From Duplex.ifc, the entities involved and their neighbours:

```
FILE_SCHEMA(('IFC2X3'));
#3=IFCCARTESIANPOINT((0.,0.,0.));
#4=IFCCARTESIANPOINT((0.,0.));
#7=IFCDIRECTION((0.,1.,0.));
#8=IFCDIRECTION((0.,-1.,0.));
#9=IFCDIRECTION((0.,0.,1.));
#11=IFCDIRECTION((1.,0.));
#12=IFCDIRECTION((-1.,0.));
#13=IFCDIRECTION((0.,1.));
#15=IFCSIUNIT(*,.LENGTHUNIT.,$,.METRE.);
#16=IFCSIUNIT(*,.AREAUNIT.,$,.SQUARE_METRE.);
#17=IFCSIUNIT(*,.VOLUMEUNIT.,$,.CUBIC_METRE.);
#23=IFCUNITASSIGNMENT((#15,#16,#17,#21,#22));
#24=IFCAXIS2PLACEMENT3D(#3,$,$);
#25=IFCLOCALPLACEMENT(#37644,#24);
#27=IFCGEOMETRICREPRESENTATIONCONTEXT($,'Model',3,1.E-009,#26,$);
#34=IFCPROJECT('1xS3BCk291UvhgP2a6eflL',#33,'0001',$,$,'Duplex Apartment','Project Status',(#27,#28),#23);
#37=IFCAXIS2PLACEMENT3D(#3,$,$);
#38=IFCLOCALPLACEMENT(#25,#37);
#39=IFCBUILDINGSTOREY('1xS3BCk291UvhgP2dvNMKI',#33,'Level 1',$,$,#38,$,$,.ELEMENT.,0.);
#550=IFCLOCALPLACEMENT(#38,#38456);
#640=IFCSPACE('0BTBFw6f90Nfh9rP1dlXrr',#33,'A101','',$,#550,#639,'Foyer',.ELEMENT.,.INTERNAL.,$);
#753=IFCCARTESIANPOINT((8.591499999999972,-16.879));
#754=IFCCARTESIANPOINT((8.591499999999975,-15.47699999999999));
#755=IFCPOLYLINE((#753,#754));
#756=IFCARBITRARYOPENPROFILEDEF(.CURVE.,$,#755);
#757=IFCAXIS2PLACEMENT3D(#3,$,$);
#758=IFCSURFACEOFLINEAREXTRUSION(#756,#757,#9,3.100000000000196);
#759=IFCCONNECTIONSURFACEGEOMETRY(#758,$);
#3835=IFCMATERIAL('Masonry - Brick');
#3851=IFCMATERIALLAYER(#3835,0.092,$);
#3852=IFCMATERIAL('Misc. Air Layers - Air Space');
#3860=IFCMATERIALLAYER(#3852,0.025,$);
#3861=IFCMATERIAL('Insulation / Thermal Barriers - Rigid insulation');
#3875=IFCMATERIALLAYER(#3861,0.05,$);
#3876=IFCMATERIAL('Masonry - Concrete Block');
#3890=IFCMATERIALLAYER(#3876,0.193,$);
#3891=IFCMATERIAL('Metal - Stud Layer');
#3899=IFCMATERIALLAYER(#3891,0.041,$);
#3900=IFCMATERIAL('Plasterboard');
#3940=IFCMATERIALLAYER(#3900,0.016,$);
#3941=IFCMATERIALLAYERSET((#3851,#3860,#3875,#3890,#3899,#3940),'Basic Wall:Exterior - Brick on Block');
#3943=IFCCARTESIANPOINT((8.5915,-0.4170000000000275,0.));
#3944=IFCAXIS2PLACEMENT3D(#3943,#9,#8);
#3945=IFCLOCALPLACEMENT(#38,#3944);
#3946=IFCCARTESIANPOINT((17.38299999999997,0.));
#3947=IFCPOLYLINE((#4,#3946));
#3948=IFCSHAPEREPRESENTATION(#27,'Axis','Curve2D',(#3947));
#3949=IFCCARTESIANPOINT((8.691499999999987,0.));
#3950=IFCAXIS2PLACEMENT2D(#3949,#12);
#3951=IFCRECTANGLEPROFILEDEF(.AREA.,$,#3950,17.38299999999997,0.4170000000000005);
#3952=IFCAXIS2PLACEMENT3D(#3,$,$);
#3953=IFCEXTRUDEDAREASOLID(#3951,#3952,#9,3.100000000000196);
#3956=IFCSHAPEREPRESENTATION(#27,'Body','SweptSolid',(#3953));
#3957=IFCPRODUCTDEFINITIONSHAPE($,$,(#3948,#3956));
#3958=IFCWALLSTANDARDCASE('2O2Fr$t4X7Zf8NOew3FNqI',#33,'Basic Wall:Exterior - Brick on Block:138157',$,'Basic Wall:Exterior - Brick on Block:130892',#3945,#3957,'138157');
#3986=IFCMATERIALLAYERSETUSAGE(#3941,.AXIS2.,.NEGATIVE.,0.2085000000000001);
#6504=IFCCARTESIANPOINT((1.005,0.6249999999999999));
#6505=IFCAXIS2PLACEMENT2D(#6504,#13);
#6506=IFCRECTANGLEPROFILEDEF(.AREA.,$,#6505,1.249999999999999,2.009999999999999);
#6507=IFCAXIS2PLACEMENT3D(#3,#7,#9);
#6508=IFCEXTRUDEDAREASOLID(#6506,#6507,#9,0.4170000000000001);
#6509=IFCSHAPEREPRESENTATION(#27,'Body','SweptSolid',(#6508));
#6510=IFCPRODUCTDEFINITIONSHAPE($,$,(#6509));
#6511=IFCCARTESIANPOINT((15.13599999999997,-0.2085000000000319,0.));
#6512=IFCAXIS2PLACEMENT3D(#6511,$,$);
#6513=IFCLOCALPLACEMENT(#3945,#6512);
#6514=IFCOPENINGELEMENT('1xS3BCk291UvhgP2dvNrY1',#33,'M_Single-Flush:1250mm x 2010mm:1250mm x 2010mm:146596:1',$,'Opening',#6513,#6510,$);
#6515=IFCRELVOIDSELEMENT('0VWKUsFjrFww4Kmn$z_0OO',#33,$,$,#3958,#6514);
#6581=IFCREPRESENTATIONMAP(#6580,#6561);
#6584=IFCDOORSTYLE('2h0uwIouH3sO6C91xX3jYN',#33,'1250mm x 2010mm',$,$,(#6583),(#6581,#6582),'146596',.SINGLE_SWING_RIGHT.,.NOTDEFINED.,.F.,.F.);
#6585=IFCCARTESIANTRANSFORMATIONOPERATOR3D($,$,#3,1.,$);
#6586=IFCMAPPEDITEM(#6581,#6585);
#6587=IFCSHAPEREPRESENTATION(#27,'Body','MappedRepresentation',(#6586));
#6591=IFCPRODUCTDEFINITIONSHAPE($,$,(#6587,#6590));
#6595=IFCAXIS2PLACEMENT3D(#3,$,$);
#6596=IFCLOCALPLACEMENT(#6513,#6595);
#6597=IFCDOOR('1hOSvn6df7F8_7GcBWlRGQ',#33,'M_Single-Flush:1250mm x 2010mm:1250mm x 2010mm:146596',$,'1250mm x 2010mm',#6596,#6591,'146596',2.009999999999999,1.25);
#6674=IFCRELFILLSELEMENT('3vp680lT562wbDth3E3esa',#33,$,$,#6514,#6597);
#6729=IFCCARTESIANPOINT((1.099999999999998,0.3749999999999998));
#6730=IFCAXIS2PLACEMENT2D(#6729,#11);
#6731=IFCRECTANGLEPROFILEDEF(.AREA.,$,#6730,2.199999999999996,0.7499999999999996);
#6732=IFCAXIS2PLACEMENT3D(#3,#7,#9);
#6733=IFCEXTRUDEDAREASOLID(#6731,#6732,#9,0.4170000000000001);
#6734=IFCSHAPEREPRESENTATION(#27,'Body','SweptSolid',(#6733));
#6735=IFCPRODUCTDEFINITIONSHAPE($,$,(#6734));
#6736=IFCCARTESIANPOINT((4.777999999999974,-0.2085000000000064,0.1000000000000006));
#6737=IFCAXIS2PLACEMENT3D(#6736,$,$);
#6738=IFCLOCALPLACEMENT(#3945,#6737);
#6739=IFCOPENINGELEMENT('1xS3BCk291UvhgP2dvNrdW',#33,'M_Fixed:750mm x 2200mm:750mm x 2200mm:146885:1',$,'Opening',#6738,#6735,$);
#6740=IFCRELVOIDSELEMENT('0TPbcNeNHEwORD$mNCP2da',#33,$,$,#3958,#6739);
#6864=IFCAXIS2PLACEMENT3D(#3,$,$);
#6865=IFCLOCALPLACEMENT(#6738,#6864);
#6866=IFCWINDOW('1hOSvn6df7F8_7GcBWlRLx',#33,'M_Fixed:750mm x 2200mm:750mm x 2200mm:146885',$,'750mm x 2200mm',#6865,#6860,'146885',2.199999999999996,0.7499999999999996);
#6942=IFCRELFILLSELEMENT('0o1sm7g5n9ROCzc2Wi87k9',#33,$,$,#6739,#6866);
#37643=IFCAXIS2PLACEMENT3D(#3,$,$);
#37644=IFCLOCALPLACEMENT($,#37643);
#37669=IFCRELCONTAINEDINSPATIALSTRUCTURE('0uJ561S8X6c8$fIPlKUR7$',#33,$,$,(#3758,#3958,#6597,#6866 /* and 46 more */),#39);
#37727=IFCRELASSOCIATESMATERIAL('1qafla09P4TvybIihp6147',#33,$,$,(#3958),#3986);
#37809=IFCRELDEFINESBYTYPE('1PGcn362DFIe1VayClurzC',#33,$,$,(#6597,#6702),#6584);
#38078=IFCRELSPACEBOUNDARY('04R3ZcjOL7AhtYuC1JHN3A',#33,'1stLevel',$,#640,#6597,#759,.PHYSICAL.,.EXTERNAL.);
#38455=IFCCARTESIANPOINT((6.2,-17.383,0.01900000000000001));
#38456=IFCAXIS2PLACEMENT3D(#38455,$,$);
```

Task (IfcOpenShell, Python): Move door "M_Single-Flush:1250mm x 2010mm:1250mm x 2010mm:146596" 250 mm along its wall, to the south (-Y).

```python
import numpy as np
import ifcopenshell
import ifcopenshell.api.geometry
import ifcopenshell.util.placement
import ifcopenshell.util.unit

model = ifcopenshell.open("Duplex.ifc")
unit_scale = ifcopenshell.util.unit.calculate_unit_scale(model)

door = model.by_id(6597)
opening = door.FillsVoids[0].RelatingOpeningElement
wall = opening.VoidsElements[0].RelatingBuildingElement

wall_matrix = ifcopenshell.util.placement.get_local_placement(wall.ObjectPlacement)
shift = wall_matrix[:3, 0] * 0.25 / unit_scale
before = ifcopenshell.util.placement.get_local_placement(door.ObjectPlacement)[:3, 3].copy()

# The door is placed relative to its opening, so it follows when the opening moves.
matrix = ifcopenshell.util.placement.get_local_placement(opening.ObjectPlacement)
matrix[:3, 3] += shift
ifcopenshell.api.geometry.edit_object_placement(
    model, product=opening, matrix=matrix, is_si=False, should_transform_children=True
)

# Space boundary surfaces are stored in each space's coordinates; move them too.
for rel in door.ProvidesBoundaries:
    if not rel.ConnectionGeometry:
        continue
    surface = rel.ConnectionGeometry.SurfaceOnRelatingElement
    space_matrix = ifcopenshell.util.placement.get_local_placement(rel.RelatingSpace.ObjectPlacement)
    point = np.array(surface.Position.Location.Coordinates) + space_matrix[:3, :3].T @ shift
    surface.Position = model.createIfcAxis2Placement3D(
        model.createIfcCartesianPoint(point.tolist()), surface.Position.Axis, surface.Position.RefDirection
    )

after = ifcopenshell.util.placement.get_local_placement(door.ObjectPlacement)[:3, 3]
print("door moved by", (after - before).round(3) + 0.0)

model.write("Duplex_rev.ifc")
```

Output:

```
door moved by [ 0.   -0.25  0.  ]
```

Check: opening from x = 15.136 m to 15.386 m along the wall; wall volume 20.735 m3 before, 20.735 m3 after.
